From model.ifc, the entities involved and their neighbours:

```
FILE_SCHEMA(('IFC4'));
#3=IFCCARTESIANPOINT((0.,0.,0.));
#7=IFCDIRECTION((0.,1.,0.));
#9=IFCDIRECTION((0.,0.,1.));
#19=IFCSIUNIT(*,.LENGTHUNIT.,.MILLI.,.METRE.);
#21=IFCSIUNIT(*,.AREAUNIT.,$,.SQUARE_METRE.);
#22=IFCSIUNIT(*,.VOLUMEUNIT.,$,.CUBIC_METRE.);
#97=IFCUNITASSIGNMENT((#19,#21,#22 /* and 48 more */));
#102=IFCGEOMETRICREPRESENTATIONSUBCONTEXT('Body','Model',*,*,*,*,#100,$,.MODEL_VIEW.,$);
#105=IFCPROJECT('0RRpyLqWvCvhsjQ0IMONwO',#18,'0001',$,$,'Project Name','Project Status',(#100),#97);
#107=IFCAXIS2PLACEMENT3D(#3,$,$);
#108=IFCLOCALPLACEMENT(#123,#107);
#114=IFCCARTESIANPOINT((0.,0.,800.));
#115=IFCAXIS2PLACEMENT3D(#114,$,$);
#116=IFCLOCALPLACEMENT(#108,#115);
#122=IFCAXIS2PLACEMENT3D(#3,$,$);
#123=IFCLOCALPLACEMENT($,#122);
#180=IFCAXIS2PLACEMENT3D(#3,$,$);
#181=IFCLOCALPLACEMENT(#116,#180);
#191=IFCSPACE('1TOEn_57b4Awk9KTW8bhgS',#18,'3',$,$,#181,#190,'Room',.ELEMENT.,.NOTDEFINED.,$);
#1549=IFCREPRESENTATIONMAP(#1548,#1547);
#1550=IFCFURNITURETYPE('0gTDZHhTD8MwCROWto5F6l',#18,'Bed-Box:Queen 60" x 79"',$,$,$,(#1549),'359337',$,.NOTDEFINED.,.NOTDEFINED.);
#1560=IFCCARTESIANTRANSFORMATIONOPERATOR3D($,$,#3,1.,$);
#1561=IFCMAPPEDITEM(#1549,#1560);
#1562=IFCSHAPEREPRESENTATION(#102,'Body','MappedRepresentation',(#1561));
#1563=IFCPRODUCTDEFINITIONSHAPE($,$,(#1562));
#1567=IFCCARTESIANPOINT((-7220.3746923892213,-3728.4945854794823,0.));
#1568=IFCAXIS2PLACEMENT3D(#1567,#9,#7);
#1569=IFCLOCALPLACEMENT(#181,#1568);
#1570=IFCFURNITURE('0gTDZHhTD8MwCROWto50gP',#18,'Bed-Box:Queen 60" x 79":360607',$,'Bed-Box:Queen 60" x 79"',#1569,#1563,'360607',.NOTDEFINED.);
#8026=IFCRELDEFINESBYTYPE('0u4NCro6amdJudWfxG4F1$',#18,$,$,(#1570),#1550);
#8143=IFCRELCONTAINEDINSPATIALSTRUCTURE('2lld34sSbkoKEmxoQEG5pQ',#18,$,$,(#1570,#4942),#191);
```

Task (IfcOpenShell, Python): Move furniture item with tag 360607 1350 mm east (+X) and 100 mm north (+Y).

```python
import ifcopenshell
import ifcopenshell.api.geometry
import ifcopenshell.util.placement
import ifcopenshell.util.unit

model = ifcopenshell.open("model.ifc")
unit_scale = ifcopenshell.util.unit.calculate_unit_scale(model)

item = model.by_guid("0gTDZHhTD8MwCROWto50gP")
matrix = ifcopenshell.util.placement.get_local_placement(item.ObjectPlacement)
matrix[0, 3] += 1.35 / unit_scale
matrix[1, 3] += 0.1 / unit_scale
ifcopenshell.api.geometry.edit_object_placement(model, product=item, matrix=matrix, is_si=False)

print(ifcopenshell.util.placement.get_local_placement(item.ObjectPlacement).round(3) + 0.0)

model.write("model_edited.ifc")
```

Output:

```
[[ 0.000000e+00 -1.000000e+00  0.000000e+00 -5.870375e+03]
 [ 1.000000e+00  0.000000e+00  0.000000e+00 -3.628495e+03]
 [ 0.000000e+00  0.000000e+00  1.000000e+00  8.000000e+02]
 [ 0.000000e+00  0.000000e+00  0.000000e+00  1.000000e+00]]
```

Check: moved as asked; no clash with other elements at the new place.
